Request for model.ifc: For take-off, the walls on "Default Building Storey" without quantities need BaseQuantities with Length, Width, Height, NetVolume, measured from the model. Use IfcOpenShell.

First a look at what the model holds.

```python
import ifcopenshell
import ifcopenshell.util.element
import ifcopenshell.util.unit

model = ifcopenshell.open("model.ifc")
print(model.schema)
for unit_type in ("LENGTHUNIT", "AREAUNIT", "VOLUMEUNIT"):
    print(unit_type, ifcopenshell.util.unit.calculate_unit_scale(model, unit_type))
storey = next(s for s in model.by_type("IfcBuildingStorey") if s.Name == "Default Building Storey")
walls = [e for e in ifcopenshell.util.element.get_decomposition(storey) if e.is_a("IfcWall")]
for e in sorted(walls, key=lambda e: e.id()):
    print(e.id(), e.is_a(), e.Name, list(ifcopenshell.util.element.get_psets(e, qtos_only=True)), sep=" | ")
```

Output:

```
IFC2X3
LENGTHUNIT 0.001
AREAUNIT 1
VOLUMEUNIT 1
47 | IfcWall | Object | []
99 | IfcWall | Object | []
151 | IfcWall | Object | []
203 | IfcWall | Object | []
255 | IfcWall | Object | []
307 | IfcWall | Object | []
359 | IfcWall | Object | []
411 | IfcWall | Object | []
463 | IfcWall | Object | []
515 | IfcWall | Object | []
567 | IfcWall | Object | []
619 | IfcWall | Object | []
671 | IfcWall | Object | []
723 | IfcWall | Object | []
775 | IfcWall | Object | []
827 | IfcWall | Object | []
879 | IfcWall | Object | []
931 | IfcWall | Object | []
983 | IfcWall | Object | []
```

```python
import ifcopenshell
import ifcopenshell.api.pset
import ifcopenshell.geom
import ifcopenshell.util.element
import ifcopenshell.util.shape
import ifcopenshell.util.unit

model = ifcopenshell.open("model.ifc")
unit_scale = ifcopenshell.util.unit.calculate_unit_scale(model)
volume_scale = ifcopenshell.util.unit.calculate_unit_scale(model, "VOLUMEUNIT")
settings = ifcopenshell.geom.settings()

storey = next(s for s in model.by_type("IfcBuildingStorey") if s.Name == "Default Building Storey")
walls = [e for e in ifcopenshell.util.element.get_decomposition(storey) if e.is_a("IfcWall")]

for e in sorted(walls, key=lambda e: e.id()):
    if ifcopenshell.util.element.get_psets(e, qtos_only=True, should_inherit=False):
        continue
    # Geometry comes back in metres, in the element's own axes.
    shape = ifcopenshell.geom.create_shape(settings, e)
    values = {
        "Length": ifcopenshell.util.shape.get_x(shape.geometry) / unit_scale,
        "Width": ifcopenshell.util.shape.get_y(shape.geometry) / unit_scale,
        "Height": ifcopenshell.util.shape.get_z(shape.geometry) / unit_scale,
        "NetVolume": ifcopenshell.util.shape.get_volume(shape.geometry) / volume_scale,
    }
    qto = ifcopenshell.api.pset.add_qto(model, product=e, name="BaseQuantities")
    ifcopenshell.api.pset.edit_qto(model, qto=qto, properties=values)
    print(e.id(), {k: round(v, 3) for k, v in values.items()})

model.write("model_v2.ifc")
```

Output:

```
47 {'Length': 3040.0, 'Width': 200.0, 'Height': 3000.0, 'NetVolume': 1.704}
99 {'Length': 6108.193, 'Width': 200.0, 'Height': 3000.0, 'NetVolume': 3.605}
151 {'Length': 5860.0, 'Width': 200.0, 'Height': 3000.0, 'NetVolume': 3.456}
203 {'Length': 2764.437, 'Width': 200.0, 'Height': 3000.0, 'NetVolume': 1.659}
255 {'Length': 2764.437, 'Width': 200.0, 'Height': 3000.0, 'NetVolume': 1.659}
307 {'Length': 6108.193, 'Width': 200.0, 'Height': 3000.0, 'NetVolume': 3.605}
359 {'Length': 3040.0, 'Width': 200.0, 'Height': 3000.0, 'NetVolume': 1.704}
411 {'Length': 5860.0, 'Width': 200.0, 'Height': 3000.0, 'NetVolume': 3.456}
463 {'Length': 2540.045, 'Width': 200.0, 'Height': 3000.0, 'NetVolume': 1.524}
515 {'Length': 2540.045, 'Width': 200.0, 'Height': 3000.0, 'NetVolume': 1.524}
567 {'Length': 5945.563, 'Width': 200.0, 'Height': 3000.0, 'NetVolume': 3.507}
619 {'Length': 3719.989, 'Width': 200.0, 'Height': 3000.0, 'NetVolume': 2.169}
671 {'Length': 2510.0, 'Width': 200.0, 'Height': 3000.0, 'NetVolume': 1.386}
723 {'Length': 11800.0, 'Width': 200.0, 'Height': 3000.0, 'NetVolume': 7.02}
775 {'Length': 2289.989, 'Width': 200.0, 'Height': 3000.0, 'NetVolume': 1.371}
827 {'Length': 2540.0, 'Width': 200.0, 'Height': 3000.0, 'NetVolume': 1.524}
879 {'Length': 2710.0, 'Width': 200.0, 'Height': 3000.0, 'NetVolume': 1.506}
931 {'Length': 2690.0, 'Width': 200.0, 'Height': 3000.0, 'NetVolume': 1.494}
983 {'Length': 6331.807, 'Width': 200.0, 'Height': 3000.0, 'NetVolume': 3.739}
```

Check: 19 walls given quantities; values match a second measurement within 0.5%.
